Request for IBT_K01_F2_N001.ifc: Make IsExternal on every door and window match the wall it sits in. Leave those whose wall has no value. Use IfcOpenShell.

First a look at what the model holds.

```python
import ifcopenshell
import ifcopenshell.util.element

model = ifcopenshell.open("IBT_K01_F2_N001.ifc")
print(model.schema)
seen = {}
for e in model.by_type("IfcDoor") + model.by_type("IfcWindow"):
    if not e.FillsVoids:
        continue
    host = e.FillsVoids[0].RelatingOpeningElement.VoidsElements[0].RelatingBuildingElement
    own = ifcopenshell.util.element.get_pset(e, f"Pset_{e.is_a()[3:].removesuffix('StandardCase')}Common", "IsExternal")
    wall = ifcopenshell.util.element.get_pset(host, "Pset_WallCommon", "IsExternal")
    seen[e.is_a(), own, wall] = seen.get((e.is_a(), own, wall), 0) + 1
for (cls, own, wall), count in sorted(seen.items(), key=str):
    print(count, cls, "IsExternal:", own, "| host wall:", wall)
```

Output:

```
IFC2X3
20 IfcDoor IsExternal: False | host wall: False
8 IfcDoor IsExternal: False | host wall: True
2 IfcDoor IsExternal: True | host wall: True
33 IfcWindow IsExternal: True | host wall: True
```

```python
import ifcopenshell
import ifcopenshell.api.pset
import ifcopenshell.util.element

model = ifcopenshell.open("IBT_K01_F2_N001.ifc")

count = 0
for ifc_class, pset_name in (("IfcDoor", "Pset_DoorCommon"), ("IfcWindow", "Pset_WindowCommon")):
    for e in model.by_type(ifc_class):
        if not e.FillsVoids:
            continue
        host = e.FillsVoids[0].RelatingOpeningElement.VoidsElements[0].RelatingBuildingElement
        external = ifcopenshell.util.element.get_pset(host, "Pset_WallCommon", "IsExternal")
        if external is None or ifcopenshell.util.element.get_pset(e, pset_name, "IsExternal") == external:
            continue
        pset = ifcopenshell.api.pset.add_pset(model, product=e, name=pset_name)
        ifcopenshell.api.pset.edit_pset(model, pset=pset, properties={"IsExternal": external})
        count += 1

print(count, "updated")

model.write("IBT_K01_F2_N001_edited.ifc")
```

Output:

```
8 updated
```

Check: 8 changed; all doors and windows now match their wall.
